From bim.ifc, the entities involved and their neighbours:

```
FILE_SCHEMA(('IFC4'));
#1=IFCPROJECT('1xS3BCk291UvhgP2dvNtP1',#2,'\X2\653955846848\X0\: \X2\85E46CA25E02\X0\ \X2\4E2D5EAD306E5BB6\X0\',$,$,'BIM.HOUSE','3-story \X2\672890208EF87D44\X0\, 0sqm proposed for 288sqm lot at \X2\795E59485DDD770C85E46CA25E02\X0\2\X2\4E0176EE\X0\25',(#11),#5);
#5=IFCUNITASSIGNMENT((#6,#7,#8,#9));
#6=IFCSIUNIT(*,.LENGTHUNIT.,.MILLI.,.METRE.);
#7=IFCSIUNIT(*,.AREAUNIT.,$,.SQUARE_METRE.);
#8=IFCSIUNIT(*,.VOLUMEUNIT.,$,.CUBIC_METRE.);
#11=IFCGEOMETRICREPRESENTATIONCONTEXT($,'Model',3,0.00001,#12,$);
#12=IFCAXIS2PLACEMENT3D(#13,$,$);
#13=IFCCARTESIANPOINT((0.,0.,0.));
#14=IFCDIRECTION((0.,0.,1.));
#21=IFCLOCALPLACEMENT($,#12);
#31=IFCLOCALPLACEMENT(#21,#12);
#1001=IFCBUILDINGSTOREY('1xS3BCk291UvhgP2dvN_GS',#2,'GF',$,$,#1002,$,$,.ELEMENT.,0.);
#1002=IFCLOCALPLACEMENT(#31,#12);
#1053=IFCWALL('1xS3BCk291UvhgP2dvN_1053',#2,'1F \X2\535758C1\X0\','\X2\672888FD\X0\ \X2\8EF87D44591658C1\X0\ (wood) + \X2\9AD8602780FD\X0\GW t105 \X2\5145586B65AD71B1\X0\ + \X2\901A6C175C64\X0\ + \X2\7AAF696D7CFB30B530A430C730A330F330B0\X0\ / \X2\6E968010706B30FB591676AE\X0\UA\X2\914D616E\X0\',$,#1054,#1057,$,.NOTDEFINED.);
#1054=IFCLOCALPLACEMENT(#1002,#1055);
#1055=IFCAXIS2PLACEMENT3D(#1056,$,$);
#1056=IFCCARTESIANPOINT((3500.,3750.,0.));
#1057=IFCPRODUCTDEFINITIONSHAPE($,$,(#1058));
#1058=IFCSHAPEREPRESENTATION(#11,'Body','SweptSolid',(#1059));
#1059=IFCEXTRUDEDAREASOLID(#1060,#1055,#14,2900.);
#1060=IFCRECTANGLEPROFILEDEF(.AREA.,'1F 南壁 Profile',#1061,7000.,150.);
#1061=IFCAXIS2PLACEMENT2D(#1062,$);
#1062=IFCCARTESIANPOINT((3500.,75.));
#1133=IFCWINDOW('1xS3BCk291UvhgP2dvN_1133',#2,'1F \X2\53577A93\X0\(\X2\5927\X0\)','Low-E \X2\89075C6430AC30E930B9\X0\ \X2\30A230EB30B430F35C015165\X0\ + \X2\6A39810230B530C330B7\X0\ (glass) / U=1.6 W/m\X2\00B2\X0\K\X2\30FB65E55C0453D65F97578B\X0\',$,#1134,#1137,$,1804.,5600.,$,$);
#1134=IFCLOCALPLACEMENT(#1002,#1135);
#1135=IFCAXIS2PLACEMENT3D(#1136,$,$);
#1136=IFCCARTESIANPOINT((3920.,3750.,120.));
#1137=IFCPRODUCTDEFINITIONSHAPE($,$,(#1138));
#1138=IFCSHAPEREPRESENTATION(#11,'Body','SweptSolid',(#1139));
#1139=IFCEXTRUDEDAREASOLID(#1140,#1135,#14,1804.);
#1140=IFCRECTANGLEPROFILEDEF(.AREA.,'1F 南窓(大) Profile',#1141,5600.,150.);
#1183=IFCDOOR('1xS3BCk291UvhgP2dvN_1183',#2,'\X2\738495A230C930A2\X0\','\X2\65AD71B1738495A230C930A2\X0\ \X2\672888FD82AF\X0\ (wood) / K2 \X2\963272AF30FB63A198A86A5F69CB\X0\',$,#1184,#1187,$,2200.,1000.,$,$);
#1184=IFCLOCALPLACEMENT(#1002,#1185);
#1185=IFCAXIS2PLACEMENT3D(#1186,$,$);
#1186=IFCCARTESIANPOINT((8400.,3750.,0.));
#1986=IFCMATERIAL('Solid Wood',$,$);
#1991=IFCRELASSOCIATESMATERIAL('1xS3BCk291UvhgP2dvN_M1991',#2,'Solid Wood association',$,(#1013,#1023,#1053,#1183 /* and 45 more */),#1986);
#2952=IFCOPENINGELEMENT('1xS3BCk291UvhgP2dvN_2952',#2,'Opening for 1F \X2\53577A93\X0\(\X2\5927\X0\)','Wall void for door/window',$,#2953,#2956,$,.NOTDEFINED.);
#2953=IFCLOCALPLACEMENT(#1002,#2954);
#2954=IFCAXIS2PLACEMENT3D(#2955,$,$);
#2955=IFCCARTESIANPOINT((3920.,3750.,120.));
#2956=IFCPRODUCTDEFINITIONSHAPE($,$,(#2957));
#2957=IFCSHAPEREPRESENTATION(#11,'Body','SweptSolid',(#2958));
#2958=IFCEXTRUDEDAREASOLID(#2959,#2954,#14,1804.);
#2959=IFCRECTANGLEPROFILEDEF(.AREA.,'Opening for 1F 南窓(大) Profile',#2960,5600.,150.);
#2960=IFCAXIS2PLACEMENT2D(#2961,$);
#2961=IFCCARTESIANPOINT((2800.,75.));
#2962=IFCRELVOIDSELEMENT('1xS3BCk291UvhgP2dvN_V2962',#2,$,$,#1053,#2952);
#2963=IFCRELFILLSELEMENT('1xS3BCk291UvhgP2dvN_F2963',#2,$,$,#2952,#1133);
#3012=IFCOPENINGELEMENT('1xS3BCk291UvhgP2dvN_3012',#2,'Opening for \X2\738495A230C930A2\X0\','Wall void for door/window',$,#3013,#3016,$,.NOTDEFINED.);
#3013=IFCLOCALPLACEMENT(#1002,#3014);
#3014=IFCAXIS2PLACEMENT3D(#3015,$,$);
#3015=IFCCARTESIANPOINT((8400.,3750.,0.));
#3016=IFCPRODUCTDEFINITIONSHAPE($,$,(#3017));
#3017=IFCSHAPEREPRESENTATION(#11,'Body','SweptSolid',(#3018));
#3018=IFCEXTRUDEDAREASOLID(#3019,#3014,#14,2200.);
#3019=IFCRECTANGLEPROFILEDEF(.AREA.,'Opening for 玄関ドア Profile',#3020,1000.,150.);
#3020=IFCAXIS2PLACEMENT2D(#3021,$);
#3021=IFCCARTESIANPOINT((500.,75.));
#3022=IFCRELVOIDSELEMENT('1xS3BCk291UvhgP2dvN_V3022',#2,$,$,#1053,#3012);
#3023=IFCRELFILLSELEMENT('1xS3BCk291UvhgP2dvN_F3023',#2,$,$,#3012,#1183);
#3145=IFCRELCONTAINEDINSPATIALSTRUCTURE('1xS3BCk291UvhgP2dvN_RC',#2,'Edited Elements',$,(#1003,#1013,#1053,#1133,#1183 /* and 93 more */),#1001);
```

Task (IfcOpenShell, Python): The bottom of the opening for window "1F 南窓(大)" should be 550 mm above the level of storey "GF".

```python
import numpy as np
import ifcopenshell
import ifcopenshell.api.geometry
import ifcopenshell.geom
import ifcopenshell.util.element
import ifcopenshell.util.placement
import ifcopenshell.util.shape
import ifcopenshell.util.unit

model = ifcopenshell.open("bim.ifc")
unit_scale = ifcopenshell.util.unit.calculate_unit_scale(model)

window = model.by_id(1133)
opening = window.FillsVoids[0].RelatingOpeningElement
storey = ifcopenshell.util.element.get_container(window, ifc_class="IfcBuildingStorey")
level = ifcopenshell.util.placement.get_local_placement(storey.ObjectPlacement)[2, 3]

# The opening's origin need not be at the sill, so measure its lowest point.
shape = ifcopenshell.geom.create_shape(ifcopenshell.geom.settings(), opening)
bottom = ifcopenshell.util.shape.get_shape_bottom_elevation(shape, shape.geometry) / unit_scale
dz = level + 0.55 / unit_scale - bottom

shift = np.array([0.0, 0.0, dz])
# The window is not placed relative to its opening, so move both.
for product in (opening, window):
    matrix = ifcopenshell.util.placement.get_local_placement(product.ObjectPlacement)
    matrix[:3, 3] += shift
    ifcopenshell.api.geometry.edit_object_placement(model, product=product, matrix=matrix, is_si=False)

print(f"moved by {dz * unit_scale:+.3f} m")

model.write("bim_updated.ifc")
```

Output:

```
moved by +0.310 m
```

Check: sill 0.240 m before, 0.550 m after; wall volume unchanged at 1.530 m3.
